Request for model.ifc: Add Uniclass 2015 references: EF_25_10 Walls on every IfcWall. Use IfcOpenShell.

First a look at what the model holds.

```python
import ifcopenshell

model = ifcopenshell.open("model.ifc")
print(model.schema)
print("classifications:", [c.Name for c in model.by_type("IfcClassification")])
for ifc_class in ("IfcDoor", "IfcRoof", "IfcStair", "IfcWall", "IfcWindow"):
    print(ifc_class, len(model.by_type(ifc_class)))
```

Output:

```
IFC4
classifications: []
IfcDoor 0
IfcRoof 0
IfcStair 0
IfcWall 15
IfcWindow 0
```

```python
import ifcopenshell
import ifcopenshell.api.classification

model = ifcopenshell.open("model.ifc")

system = ifcopenshell.api.classification.add_classification(model, classification="Uniclass 2015")

codes = {
    "IfcWall": ("EF_25_10", "Walls"),
}
for ifc_class, (code, name) in codes.items():
    products = model.by_type(ifc_class)
    ifcopenshell.api.classification.add_reference(
        model, products=products, classification=system, identification=code, name=name
    )
    print(code, len(products))

model.write("model_updated.ifc")
```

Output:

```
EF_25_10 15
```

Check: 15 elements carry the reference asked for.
